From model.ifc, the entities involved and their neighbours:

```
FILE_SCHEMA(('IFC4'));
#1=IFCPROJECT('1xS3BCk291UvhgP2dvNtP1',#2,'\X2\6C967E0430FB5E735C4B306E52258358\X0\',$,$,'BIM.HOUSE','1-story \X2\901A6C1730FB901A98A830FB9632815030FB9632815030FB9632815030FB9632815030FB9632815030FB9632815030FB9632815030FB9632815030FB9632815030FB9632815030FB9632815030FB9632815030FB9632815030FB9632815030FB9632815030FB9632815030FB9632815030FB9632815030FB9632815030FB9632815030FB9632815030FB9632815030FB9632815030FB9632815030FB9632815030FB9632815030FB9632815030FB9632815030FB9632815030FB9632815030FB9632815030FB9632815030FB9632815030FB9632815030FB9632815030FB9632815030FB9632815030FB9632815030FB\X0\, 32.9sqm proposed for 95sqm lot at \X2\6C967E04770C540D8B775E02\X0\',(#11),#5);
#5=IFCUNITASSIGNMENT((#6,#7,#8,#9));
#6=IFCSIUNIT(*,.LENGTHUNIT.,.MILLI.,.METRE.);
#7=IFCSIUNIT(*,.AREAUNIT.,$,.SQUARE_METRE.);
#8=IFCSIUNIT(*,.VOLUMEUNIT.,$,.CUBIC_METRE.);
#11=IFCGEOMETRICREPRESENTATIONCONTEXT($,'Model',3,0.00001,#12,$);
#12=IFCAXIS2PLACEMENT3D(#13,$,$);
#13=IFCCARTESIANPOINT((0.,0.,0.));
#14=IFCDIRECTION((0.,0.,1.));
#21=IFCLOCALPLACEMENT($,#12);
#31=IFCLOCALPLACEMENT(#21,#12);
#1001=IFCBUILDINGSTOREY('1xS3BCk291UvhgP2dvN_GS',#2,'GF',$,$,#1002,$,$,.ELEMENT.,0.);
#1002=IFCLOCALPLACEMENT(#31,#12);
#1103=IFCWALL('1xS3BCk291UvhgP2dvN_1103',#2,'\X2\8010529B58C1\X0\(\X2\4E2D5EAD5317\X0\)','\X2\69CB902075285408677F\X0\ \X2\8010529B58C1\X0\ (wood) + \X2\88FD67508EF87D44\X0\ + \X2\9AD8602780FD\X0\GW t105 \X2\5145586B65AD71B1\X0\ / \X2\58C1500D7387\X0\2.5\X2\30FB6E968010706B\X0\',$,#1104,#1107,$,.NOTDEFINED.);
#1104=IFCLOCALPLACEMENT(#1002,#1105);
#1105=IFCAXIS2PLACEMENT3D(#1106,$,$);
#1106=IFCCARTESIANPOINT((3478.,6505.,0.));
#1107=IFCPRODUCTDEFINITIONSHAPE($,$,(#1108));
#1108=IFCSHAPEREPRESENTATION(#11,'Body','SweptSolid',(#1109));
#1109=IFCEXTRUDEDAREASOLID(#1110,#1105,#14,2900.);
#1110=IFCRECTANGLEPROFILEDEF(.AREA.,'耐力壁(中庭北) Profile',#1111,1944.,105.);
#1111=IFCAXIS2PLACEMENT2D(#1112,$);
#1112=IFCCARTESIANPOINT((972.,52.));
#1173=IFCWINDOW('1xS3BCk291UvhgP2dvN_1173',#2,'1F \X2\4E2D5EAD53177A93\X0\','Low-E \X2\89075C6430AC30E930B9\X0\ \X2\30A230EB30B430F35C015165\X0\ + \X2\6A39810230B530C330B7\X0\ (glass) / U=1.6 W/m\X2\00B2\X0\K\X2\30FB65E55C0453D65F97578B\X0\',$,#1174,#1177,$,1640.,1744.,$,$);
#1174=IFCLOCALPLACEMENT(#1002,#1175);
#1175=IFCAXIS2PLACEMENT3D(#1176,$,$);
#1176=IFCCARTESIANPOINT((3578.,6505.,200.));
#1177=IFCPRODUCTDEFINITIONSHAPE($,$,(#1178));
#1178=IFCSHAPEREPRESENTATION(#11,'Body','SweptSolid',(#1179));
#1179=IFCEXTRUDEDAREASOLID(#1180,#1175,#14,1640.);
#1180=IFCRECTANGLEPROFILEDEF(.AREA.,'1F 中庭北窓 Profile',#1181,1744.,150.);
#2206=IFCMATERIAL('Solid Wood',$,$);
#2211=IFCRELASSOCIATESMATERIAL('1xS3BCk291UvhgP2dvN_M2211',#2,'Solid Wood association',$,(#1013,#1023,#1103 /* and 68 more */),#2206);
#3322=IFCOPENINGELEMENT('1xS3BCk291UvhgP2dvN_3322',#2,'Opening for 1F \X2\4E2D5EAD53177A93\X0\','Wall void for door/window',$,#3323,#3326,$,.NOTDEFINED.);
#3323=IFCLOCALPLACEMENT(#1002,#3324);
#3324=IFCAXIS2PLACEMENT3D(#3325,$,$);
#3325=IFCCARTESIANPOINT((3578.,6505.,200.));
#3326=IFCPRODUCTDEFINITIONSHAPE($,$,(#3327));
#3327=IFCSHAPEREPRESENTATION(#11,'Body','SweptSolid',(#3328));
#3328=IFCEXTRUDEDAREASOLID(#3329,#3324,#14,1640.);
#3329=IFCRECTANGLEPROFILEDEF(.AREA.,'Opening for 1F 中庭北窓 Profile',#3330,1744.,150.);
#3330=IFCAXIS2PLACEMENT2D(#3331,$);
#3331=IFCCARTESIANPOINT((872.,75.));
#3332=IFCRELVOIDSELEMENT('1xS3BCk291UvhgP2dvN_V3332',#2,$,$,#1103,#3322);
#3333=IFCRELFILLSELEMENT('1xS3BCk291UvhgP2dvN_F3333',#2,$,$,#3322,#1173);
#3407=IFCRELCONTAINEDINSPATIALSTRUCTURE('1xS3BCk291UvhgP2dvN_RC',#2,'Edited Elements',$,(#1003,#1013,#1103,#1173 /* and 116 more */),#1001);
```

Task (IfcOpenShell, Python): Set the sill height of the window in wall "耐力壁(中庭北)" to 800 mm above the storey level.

```python
import numpy as np
import ifcopenshell
import ifcopenshell.api.geometry
import ifcopenshell.geom
import ifcopenshell.util.element
import ifcopenshell.util.placement
import ifcopenshell.util.shape
import ifcopenshell.util.unit

model = ifcopenshell.open("model.ifc")
unit_scale = ifcopenshell.util.unit.calculate_unit_scale(model)

window = model.by_guid("1xS3BCk291UvhgP2dvN_1173")
opening = window.FillsVoids[0].RelatingOpeningElement
storey = ifcopenshell.util.element.get_container(window, ifc_class="IfcBuildingStorey")
level = ifcopenshell.util.placement.get_local_placement(storey.ObjectPlacement)[2, 3]

# The opening's origin need not be at the sill, so measure its lowest point.
shape = ifcopenshell.geom.create_shape(ifcopenshell.geom.settings(), opening)
bottom = ifcopenshell.util.shape.get_shape_bottom_elevation(shape, shape.geometry) / unit_scale
dz = level + 0.8 / unit_scale - bottom

shift = np.array([0.0, 0.0, dz])
# The window is not placed relative to its opening, so move both.
for product in (opening, window):
    matrix = ifcopenshell.util.placement.get_local_placement(product.ObjectPlacement)
    matrix[:3, 3] += shift
    ifcopenshell.api.geometry.edit_object_placement(model, product=product, matrix=matrix, is_si=False)

print(f"moved by {dz * unit_scale:+.3f} m")

model.write("model_edited.ifc")
```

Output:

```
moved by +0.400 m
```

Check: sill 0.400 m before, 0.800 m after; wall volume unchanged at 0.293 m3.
